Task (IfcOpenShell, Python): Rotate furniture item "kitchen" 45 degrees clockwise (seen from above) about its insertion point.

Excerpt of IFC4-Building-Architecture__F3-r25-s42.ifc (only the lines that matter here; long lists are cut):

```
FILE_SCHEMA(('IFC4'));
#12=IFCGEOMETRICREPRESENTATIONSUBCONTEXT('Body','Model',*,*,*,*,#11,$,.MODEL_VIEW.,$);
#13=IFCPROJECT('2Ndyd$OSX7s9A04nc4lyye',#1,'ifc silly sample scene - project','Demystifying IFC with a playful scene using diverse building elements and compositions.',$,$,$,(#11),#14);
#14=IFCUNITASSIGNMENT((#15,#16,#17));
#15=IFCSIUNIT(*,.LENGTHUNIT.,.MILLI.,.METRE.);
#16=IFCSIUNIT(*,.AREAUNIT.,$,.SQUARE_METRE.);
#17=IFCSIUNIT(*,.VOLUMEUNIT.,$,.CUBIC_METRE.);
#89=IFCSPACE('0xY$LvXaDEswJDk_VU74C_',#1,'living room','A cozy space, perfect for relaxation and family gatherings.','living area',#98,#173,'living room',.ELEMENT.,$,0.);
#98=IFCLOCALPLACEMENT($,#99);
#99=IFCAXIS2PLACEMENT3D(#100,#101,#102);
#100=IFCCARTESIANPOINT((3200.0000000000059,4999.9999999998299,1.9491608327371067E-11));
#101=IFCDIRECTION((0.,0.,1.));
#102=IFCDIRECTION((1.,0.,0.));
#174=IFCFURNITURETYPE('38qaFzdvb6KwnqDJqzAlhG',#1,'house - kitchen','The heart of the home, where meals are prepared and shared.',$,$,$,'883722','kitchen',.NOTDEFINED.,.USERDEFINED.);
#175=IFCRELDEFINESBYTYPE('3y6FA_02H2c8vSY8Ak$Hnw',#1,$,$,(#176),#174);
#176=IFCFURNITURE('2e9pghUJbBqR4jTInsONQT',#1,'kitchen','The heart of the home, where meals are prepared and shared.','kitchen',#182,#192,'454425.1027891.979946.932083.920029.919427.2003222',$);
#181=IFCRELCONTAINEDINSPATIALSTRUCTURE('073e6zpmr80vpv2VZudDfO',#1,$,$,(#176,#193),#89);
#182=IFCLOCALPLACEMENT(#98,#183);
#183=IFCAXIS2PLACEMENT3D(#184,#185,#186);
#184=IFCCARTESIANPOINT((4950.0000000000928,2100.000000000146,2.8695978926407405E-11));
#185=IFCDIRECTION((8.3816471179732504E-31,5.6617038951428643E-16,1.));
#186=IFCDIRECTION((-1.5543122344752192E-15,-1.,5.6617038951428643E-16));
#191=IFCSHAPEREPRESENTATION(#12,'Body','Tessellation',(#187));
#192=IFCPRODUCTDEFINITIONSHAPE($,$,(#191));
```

```python
import ifcopenshell
import ifcopenshell.api.geometry
import ifcopenshell.util.placement

model = ifcopenshell.open("IFC4-Building-Architecture__F3-r25-s42.ifc")

item = model.by_guid("2e9pghUJbBqR4jTInsONQT")
matrix = ifcopenshell.util.placement.get_local_placement(item.ObjectPlacement)
matrix = matrix @ ifcopenshell.util.placement.rotation(-45, "Z")
ifcopenshell.api.geometry.edit_object_placement(model, product=item, matrix=matrix, is_si=False)

print(ifcopenshell.util.placement.get_local_placement(item.ObjectPlacement).round(3) + 0.0)

model.write("IFC4-Building-Architecture__F3-r25-s42_updated.ifc")
```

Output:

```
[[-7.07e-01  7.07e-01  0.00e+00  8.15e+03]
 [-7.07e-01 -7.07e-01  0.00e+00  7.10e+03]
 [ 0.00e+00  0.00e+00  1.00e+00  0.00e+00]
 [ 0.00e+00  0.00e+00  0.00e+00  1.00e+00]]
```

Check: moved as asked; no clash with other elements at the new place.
